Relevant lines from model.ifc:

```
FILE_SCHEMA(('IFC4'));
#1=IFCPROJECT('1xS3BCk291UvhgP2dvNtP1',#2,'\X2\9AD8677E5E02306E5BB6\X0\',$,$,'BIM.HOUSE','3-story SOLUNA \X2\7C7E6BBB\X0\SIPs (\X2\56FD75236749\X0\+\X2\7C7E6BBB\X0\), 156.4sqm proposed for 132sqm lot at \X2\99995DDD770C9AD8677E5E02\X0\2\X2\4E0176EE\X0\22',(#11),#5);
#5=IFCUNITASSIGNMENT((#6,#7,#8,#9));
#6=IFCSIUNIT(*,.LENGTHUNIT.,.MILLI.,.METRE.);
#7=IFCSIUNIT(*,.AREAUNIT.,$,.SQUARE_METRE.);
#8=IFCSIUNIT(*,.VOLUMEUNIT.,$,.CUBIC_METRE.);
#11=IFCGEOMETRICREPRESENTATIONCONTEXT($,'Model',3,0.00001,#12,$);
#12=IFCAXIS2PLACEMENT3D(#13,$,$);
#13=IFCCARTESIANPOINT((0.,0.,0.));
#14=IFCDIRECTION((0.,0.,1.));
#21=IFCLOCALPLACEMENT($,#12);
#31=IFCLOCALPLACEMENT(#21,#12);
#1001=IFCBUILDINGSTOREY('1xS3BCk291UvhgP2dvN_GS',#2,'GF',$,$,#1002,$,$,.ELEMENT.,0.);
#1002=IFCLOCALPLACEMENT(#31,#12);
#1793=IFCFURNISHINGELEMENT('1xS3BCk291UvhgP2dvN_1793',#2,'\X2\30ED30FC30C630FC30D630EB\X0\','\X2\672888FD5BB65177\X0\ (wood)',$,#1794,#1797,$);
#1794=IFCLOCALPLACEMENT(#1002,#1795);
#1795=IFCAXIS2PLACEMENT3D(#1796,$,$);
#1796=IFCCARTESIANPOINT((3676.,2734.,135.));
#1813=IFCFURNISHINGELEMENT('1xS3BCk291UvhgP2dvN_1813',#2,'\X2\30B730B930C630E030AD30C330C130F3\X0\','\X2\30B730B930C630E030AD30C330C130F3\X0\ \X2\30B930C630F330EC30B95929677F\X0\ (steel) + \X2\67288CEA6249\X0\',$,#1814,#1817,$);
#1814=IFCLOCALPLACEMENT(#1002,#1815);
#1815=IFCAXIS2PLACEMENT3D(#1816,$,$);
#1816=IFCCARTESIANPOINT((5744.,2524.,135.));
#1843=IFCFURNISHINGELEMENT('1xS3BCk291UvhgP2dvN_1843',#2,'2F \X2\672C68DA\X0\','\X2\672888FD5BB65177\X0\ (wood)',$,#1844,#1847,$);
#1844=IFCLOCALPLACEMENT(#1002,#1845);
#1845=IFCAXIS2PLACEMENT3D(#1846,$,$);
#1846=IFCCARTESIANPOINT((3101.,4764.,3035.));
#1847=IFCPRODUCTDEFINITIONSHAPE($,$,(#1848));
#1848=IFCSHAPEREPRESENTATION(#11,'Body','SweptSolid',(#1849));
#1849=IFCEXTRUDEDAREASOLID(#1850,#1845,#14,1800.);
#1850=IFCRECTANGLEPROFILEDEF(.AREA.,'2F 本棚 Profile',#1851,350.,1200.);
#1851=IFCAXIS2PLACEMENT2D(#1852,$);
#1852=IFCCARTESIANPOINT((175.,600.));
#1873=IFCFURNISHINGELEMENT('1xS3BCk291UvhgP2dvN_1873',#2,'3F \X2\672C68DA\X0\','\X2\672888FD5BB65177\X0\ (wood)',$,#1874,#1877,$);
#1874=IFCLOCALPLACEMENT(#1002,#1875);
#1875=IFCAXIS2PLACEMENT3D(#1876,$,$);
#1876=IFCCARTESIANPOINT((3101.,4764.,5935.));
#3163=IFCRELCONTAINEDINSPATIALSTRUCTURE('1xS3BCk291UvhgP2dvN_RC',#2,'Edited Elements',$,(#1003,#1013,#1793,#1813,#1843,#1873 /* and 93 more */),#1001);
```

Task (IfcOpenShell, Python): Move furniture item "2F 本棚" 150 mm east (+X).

```python
import ifcopenshell
import ifcopenshell.api.geometry
import ifcopenshell.util.placement
import ifcopenshell.util.unit

model = ifcopenshell.open("model.ifc")
unit_scale = ifcopenshell.util.unit.calculate_unit_scale(model)

item = model.by_guid("1xS3BCk291UvhgP2dvN_1843")
matrix = ifcopenshell.util.placement.get_local_placement(item.ObjectPlacement)
matrix[0, 3] += 0.15 / unit_scale
ifcopenshell.api.geometry.edit_object_placement(model, product=item, matrix=matrix, is_si=False)

print(ifcopenshell.util.placement.get_local_placement(item.ObjectPlacement).round(3) + 0.0)

model.write("model_rev.ifc")
```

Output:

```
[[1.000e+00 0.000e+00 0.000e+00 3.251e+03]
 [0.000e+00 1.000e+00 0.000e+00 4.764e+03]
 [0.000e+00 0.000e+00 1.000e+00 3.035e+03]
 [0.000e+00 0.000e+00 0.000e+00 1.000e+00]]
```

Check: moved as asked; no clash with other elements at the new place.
